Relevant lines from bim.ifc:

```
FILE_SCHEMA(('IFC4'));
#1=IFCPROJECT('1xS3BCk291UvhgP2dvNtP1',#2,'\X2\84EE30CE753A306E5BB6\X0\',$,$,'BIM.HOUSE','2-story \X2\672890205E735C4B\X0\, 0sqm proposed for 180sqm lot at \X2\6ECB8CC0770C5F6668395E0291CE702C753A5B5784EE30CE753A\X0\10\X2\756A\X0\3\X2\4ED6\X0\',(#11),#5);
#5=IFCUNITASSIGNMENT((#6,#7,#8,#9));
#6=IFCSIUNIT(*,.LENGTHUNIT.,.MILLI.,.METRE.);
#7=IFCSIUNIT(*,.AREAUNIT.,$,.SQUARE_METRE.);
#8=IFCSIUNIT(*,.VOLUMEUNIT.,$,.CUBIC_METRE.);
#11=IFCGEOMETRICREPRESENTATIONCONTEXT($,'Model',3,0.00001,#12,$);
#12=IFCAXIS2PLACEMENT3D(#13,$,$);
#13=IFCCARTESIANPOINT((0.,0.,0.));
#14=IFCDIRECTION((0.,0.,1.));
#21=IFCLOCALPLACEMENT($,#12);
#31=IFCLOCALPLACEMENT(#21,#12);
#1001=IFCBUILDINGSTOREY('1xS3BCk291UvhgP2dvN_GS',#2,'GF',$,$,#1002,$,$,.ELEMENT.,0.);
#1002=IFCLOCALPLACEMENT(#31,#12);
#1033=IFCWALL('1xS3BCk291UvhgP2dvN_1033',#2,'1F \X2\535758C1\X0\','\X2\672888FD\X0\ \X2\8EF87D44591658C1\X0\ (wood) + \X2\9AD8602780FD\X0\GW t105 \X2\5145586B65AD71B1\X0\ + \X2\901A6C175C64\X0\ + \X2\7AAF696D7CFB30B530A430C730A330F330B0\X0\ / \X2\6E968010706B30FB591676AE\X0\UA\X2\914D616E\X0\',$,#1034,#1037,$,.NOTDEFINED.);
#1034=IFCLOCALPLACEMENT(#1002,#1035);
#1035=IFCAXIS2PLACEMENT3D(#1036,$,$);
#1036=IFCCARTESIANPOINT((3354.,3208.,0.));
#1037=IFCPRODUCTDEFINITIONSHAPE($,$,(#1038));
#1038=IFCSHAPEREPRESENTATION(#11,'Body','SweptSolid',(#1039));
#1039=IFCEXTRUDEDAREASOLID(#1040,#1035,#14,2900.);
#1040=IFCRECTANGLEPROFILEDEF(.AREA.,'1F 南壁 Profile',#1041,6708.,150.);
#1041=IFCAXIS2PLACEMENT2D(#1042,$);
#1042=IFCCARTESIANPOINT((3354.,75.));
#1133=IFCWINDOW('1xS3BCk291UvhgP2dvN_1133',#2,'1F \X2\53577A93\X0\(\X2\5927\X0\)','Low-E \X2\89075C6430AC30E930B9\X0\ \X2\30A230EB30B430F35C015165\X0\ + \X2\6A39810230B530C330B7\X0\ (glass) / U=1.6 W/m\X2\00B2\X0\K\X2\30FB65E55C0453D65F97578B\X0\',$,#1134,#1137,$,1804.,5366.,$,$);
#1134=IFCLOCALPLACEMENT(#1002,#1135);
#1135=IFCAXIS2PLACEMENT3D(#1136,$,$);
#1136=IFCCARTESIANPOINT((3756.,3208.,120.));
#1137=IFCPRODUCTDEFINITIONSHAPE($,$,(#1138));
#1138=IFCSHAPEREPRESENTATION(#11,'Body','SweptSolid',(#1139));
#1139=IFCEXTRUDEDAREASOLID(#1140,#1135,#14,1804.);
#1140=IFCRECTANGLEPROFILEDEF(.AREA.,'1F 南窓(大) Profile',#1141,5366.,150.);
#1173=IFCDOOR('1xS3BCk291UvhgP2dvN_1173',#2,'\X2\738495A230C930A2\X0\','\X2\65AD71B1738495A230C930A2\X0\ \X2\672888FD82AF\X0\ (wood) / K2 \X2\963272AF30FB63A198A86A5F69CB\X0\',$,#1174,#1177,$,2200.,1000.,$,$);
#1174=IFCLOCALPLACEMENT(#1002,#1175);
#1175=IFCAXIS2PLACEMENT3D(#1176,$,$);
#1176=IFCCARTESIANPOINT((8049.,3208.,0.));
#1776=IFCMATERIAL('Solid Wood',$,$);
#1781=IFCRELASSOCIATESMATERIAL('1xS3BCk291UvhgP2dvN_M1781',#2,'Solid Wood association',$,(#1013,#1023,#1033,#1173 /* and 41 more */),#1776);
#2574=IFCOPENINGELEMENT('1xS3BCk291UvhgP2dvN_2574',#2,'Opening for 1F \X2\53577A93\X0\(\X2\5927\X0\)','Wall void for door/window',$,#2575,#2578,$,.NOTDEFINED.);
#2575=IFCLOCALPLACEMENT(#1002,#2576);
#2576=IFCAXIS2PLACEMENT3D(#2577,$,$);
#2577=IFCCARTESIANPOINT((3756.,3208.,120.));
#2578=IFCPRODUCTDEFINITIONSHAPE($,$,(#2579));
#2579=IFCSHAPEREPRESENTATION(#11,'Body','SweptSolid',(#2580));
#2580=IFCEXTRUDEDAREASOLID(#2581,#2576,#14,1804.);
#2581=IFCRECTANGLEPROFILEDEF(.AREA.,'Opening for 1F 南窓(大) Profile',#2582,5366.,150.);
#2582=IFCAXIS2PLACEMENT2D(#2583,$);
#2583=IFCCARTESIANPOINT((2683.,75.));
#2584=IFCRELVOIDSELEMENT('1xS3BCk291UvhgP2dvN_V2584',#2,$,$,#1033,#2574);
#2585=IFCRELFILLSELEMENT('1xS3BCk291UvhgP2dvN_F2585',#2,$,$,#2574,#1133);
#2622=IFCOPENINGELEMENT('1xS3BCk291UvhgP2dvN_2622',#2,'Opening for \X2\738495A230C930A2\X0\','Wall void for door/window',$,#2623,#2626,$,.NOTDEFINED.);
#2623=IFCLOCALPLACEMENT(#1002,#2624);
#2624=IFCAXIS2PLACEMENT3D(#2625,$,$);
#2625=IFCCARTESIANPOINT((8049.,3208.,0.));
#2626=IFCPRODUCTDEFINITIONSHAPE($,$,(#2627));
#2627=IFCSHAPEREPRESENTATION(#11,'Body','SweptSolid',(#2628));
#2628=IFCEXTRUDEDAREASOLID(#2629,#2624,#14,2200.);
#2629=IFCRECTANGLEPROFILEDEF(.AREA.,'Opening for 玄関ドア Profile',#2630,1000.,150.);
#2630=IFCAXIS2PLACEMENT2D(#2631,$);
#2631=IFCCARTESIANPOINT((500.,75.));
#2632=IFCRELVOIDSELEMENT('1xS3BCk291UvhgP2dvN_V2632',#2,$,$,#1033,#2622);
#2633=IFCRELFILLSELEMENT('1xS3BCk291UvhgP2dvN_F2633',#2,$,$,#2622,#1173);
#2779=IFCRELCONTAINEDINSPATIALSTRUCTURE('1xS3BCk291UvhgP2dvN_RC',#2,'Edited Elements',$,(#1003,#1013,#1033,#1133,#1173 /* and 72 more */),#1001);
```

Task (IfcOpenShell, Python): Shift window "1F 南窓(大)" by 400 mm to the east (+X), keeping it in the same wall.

```python
import ifcopenshell
import ifcopenshell.api.geometry
import ifcopenshell.util.placement
import ifcopenshell.util.unit

model = ifcopenshell.open("bim.ifc")
unit_scale = ifcopenshell.util.unit.calculate_unit_scale(model)

window = model.by_id(1133)
opening = window.FillsVoids[0].RelatingOpeningElement
wall = opening.VoidsElements[0].RelatingBuildingElement

wall_matrix = ifcopenshell.util.placement.get_local_placement(wall.ObjectPlacement)
shift = wall_matrix[:3, 0] * 0.4 / unit_scale
before = ifcopenshell.util.placement.get_local_placement(window.ObjectPlacement)[:3, 3].copy()

# The window is not placed relative to its opening, so move both.
for product in (opening, window):
    matrix = ifcopenshell.util.placement.get_local_placement(product.ObjectPlacement)
    matrix[:3, 3] += shift
    ifcopenshell.api.geometry.edit_object_placement(model, product=product, matrix=matrix, is_si=False)

after = ifcopenshell.util.placement.get_local_placement(window.ObjectPlacement)[:3, 3]
print("window moved by", (after - before).round(3) + 0.0)

model.write("bim_updated.ifc")
```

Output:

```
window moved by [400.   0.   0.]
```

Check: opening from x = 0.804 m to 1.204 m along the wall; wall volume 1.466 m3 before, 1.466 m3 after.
